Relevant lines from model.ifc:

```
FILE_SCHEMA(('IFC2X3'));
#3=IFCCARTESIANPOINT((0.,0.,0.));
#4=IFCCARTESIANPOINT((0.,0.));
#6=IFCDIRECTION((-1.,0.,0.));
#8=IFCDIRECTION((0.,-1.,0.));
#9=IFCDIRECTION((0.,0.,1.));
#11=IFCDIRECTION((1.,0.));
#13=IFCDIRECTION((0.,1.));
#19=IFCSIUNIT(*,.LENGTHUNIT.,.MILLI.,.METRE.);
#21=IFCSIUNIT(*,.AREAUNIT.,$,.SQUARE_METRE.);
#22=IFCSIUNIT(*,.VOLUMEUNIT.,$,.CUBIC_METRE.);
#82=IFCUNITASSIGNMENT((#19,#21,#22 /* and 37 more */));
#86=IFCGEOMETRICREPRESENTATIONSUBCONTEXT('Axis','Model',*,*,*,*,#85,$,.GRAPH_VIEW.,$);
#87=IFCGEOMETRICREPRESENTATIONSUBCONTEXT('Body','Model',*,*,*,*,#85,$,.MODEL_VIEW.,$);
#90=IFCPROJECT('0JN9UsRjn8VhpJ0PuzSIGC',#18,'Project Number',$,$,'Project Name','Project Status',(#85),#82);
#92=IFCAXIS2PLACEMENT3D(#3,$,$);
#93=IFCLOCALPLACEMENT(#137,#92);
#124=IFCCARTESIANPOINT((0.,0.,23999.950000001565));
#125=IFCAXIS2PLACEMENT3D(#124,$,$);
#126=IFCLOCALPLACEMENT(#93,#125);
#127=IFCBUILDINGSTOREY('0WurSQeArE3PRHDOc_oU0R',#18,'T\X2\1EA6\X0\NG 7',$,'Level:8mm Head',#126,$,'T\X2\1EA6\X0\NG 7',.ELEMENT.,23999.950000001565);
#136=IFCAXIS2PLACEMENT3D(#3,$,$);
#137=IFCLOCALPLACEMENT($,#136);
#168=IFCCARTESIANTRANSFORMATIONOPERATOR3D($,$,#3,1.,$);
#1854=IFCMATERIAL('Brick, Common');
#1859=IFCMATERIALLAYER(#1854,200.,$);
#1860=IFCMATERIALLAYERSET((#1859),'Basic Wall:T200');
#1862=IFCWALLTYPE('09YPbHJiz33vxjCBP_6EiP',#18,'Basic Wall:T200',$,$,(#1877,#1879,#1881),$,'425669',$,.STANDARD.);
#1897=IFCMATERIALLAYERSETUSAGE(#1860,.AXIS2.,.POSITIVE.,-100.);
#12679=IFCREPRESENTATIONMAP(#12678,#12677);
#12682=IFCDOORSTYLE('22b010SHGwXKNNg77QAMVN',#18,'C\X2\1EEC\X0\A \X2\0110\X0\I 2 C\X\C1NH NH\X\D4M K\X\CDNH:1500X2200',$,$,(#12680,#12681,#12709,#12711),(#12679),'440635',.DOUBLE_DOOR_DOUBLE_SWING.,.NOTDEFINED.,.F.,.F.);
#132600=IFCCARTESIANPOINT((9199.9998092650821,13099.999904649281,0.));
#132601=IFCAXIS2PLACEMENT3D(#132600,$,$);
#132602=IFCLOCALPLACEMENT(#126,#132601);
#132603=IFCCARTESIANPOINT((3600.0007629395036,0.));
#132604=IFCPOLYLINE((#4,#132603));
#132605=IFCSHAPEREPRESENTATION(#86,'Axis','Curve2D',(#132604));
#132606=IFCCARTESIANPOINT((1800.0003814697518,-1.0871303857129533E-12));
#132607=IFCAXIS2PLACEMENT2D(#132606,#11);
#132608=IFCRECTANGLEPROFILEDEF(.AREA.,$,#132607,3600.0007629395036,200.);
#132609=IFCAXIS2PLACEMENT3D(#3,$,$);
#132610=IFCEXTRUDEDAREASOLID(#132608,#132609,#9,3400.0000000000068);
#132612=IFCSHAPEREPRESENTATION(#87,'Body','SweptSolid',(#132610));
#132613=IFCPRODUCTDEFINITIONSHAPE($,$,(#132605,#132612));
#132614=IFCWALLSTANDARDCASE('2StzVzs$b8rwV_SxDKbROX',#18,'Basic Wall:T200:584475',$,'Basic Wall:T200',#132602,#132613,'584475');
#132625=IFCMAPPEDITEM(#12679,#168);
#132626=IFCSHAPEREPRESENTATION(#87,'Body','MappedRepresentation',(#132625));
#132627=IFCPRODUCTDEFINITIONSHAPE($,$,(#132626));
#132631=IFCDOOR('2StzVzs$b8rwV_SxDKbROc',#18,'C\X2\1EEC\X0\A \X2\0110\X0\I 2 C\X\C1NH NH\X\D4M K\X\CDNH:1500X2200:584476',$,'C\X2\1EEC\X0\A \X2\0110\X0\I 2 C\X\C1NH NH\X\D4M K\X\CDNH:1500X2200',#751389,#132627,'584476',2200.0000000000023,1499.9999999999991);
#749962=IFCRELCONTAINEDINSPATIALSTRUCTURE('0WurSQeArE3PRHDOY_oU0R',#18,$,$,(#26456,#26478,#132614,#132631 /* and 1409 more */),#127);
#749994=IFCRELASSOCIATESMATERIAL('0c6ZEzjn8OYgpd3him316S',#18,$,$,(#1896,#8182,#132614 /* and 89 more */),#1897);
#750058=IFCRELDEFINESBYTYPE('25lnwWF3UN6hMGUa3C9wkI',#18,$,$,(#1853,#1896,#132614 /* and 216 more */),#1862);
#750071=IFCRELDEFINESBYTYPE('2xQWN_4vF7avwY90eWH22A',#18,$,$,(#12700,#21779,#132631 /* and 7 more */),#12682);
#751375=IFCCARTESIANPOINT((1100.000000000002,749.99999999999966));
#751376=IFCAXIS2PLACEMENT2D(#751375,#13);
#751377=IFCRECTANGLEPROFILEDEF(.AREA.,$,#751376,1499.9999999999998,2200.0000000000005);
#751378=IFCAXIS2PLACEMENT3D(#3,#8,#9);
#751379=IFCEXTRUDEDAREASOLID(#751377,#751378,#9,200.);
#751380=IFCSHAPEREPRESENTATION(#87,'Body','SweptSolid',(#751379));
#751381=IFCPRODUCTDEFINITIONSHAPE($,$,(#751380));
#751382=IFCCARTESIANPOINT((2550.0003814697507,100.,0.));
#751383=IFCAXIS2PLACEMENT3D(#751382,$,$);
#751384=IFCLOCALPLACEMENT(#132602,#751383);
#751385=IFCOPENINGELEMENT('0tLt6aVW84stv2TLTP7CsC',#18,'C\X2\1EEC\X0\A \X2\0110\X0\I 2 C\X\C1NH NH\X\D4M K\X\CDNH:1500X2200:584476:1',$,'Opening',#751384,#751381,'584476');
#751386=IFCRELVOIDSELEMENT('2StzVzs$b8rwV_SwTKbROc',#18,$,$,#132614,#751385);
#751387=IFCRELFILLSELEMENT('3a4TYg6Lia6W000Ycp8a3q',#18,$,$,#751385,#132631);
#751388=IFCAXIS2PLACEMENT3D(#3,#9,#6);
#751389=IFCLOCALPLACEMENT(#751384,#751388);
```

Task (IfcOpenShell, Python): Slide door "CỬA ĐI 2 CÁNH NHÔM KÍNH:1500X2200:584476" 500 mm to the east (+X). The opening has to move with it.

```python
import ifcopenshell
import ifcopenshell.api.geometry
import ifcopenshell.util.placement
import ifcopenshell.util.unit

model = ifcopenshell.open("model.ifc")
unit_scale = ifcopenshell.util.unit.calculate_unit_scale(model)

door = model.by_id(132631)
opening = door.FillsVoids[0].RelatingOpeningElement
wall = opening.VoidsElements[0].RelatingBuildingElement

wall_matrix = ifcopenshell.util.placement.get_local_placement(wall.ObjectPlacement)
shift = wall_matrix[:3, 0] * 0.5 / unit_scale
before = ifcopenshell.util.placement.get_local_placement(door.ObjectPlacement)[:3, 3].copy()

# The door is placed relative to its opening, so it follows when the opening moves.
matrix = ifcopenshell.util.placement.get_local_placement(opening.ObjectPlacement)
matrix[:3, 3] += shift
ifcopenshell.api.geometry.edit_object_placement(
    model, product=opening, matrix=matrix, is_si=False, should_transform_children=True
)

after = ifcopenshell.util.placement.get_local_placement(door.ObjectPlacement)[:3, 3]
print("door moved by", (after - before).round(3) + 0.0)

model.write("model_edited.ifc")
```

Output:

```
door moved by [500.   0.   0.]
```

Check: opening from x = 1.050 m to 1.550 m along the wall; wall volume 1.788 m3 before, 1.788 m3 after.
